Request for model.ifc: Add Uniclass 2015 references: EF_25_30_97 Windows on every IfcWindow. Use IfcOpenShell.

First a look at what the model holds.

```python
import ifcopenshell

model = ifcopenshell.open("model.ifc")
print(model.schema)
print("classifications:", [c.Name for c in model.by_type("IfcClassification")])
for ifc_class in ("IfcDoor", "IfcRoof", "IfcStair", "IfcWall", "IfcWindow"):
    print(ifc_class, len(model.by_type(ifc_class)))
```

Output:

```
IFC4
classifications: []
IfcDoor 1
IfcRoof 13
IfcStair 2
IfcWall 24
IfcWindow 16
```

```python
import ifcopenshell
import ifcopenshell.api.classification

model = ifcopenshell.open("model.ifc")

system = ifcopenshell.api.classification.add_classification(model, classification="Uniclass 2015")

codes = {
    "IfcWindow": ("EF_25_30_97", "Windows"),
}
for ifc_class, (code, name) in codes.items():
    products = model.by_type(ifc_class)
    ifcopenshell.api.classification.add_reference(
        model, products=products, classification=system, identification=code, name=name
    )
    print(code, len(products))

model.write("model_rev.ifc")
```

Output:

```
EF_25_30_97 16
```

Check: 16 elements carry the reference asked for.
